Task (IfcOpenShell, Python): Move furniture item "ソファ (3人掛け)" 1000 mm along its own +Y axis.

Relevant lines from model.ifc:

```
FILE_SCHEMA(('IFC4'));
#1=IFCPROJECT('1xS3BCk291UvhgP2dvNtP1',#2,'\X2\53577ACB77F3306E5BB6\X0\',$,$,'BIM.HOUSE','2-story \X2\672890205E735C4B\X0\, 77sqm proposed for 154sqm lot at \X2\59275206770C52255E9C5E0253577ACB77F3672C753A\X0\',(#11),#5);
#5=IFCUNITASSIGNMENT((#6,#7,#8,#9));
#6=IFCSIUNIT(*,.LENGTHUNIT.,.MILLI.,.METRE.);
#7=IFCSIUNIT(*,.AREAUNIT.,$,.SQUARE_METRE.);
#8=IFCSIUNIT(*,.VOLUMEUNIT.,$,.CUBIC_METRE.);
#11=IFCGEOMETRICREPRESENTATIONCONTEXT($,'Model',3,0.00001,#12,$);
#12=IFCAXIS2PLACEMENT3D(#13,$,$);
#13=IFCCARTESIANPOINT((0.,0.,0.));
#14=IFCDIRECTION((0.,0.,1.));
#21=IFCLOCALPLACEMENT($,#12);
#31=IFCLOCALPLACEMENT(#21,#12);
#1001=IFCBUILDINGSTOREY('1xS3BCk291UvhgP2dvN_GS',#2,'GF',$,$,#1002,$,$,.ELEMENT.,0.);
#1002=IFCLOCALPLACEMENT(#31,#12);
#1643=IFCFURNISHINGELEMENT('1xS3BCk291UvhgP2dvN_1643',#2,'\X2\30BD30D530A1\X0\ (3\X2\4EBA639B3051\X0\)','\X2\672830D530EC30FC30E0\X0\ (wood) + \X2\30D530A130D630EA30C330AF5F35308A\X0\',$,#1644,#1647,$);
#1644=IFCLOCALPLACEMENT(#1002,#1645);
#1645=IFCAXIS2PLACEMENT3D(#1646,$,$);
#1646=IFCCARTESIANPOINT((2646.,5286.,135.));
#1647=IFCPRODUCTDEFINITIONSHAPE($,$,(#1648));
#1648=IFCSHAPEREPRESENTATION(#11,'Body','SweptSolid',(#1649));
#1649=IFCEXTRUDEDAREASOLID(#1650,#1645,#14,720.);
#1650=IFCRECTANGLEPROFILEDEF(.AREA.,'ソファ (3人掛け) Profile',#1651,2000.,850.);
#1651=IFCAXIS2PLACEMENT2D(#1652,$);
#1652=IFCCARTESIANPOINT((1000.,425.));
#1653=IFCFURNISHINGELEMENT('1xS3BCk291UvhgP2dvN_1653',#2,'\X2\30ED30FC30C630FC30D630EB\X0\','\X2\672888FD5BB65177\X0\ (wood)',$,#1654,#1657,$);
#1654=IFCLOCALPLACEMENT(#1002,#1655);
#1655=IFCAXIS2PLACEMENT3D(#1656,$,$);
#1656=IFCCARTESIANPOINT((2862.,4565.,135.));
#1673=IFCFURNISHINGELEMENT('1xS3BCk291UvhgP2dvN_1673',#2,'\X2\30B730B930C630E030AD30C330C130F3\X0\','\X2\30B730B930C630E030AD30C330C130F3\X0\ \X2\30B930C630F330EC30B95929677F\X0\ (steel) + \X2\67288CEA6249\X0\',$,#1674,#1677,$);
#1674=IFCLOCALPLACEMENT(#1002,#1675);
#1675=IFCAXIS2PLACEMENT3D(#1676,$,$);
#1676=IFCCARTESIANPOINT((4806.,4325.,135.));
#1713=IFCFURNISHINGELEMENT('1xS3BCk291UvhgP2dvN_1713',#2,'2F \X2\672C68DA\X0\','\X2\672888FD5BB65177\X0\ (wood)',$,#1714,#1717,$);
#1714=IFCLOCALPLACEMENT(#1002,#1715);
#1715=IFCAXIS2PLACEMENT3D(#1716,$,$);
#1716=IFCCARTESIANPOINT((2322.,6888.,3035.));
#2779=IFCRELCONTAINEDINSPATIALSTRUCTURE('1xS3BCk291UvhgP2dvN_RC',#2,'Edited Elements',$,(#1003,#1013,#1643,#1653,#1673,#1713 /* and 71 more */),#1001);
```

```python
import ifcopenshell
import ifcopenshell.api.geometry
import ifcopenshell.util.placement
import ifcopenshell.util.unit

model = ifcopenshell.open("model.ifc")
unit_scale = ifcopenshell.util.unit.calculate_unit_scale(model)

item = model.by_id(1643)
matrix = ifcopenshell.util.placement.get_local_placement(item.ObjectPlacement)
matrix[:3, 3] += matrix[:3, 1] * 1 / unit_scale
ifcopenshell.api.geometry.edit_object_placement(model, product=item, matrix=matrix, is_si=False)

print(ifcopenshell.util.placement.get_local_placement(item.ObjectPlacement).round(3) + 0.0)

model.write("model_rev.ifc")
```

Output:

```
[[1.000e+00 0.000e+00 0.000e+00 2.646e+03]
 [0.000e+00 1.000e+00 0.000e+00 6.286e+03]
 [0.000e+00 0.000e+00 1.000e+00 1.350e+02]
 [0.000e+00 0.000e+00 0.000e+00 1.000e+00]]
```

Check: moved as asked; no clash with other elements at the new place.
